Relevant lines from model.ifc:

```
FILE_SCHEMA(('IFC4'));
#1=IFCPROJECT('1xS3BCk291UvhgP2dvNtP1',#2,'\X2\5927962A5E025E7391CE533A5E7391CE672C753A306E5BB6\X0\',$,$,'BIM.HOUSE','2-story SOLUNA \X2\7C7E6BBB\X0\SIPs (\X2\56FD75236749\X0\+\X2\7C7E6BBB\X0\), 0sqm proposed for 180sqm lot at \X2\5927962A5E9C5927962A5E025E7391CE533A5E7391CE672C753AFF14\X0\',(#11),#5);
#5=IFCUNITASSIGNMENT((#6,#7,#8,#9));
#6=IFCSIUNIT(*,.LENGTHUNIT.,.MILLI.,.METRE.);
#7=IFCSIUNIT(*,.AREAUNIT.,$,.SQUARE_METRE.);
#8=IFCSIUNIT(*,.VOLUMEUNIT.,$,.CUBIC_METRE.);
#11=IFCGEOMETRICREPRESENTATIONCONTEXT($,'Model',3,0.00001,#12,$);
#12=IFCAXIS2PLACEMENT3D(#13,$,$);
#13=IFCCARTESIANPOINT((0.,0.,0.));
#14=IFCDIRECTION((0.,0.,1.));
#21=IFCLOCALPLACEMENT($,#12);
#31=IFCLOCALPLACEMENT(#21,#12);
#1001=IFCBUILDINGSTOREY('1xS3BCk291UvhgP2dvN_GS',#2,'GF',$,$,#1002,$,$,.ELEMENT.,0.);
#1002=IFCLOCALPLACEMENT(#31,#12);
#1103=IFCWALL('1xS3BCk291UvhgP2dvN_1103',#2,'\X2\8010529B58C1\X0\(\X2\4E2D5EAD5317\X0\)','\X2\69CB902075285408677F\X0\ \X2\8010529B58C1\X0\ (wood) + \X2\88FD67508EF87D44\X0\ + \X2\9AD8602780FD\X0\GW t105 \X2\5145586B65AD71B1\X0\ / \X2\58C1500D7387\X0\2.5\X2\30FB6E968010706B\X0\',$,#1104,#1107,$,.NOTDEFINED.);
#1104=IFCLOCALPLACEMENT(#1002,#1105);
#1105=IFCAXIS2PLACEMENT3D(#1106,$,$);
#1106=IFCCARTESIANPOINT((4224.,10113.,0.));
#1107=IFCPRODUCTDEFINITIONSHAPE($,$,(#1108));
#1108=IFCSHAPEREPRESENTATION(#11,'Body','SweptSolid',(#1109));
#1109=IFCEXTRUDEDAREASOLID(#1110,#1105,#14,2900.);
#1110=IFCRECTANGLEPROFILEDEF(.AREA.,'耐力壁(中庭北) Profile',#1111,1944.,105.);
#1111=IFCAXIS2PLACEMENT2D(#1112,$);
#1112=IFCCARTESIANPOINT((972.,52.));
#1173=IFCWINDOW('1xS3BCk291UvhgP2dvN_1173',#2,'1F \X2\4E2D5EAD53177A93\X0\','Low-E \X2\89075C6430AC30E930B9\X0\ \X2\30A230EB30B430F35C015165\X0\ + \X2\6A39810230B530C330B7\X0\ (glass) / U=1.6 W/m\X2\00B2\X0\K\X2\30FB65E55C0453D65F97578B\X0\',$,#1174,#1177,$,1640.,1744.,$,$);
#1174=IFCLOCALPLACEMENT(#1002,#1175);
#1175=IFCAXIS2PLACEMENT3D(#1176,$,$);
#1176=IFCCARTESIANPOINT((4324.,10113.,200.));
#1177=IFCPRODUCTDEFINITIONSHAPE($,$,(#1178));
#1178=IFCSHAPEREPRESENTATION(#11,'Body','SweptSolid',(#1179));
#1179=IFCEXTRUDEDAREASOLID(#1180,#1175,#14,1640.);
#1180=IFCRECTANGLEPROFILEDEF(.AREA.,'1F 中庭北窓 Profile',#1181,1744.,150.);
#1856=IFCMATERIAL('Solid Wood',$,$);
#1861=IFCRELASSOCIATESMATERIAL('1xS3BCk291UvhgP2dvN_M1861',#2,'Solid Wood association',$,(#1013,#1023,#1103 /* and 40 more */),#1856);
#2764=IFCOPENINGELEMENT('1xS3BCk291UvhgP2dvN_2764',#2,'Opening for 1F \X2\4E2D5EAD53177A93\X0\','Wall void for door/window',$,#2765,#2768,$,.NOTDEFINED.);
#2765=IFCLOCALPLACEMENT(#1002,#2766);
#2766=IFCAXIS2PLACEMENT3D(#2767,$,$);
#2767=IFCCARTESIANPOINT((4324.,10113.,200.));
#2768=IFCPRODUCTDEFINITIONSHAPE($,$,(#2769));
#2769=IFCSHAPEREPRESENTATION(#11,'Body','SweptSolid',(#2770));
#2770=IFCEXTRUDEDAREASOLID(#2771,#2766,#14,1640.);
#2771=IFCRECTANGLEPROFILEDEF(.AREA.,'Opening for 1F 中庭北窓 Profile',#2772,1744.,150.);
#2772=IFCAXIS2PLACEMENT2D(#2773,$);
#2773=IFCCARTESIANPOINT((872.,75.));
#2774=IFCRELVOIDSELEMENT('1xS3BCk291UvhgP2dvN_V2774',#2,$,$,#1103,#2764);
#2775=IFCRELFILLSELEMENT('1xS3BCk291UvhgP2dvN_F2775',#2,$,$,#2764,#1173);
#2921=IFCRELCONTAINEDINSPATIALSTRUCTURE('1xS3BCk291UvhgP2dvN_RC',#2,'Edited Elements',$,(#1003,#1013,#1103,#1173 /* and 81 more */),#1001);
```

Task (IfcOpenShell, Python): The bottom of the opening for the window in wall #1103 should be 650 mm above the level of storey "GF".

```python
import numpy as np
import ifcopenshell
import ifcopenshell.api.geometry
import ifcopenshell.geom
import ifcopenshell.util.element
import ifcopenshell.util.placement
import ifcopenshell.util.shape
import ifcopenshell.util.unit

model = ifcopenshell.open("model.ifc")
unit_scale = ifcopenshell.util.unit.calculate_unit_scale(model)

window = model.by_id(1173)
opening = window.FillsVoids[0].RelatingOpeningElement
storey = ifcopenshell.util.element.get_container(window, ifc_class="IfcBuildingStorey")
level = ifcopenshell.util.placement.get_local_placement(storey.ObjectPlacement)[2, 3]

# The opening's origin need not be at the sill, so measure its lowest point.
shape = ifcopenshell.geom.create_shape(ifcopenshell.geom.settings(), opening)
bottom = ifcopenshell.util.shape.get_shape_bottom_elevation(shape, shape.geometry) / unit_scale
dz = level + 650.0 - bottom

shift = np.array([0.0, 0.0, dz])
# The window is not placed relative to its opening, so move both.
for product in (opening, window):
    matrix = ifcopenshell.util.placement.get_local_placement(product.ObjectPlacement)
    matrix[:3, 3] += shift
    ifcopenshell.api.geometry.edit_object_placement(model, product=product, matrix=matrix, is_si=False)

print(f"moved by {dz * unit_scale:+.3f} m")

model.write("model_edited.ifc")
```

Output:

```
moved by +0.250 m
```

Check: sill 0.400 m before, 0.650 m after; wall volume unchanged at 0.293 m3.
